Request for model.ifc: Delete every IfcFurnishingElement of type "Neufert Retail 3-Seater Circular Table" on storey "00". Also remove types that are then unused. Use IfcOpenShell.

First a look at what the model holds.

```python
import ifcopenshell
import ifcopenshell.util.element

model = ifcopenshell.open("model.ifc")
print(model.schema)
storey = next(s for s in model.by_type("IfcBuildingStorey") if s.Name == "00")
furniture = [e for e in ifcopenshell.util.element.get_decomposition(storey) if e.is_a("IfcFurnishingElement")]
seen = {}
for e in furniture:
    element_type = ifcopenshell.util.element.get_type(e)
    name = element_type.Name if element_type not in (None, e) else None
    seen[name] = seen.get(name, 0) + 1
for name, count in sorted(seen.items(), key=str):
    print(count, "x", name)
```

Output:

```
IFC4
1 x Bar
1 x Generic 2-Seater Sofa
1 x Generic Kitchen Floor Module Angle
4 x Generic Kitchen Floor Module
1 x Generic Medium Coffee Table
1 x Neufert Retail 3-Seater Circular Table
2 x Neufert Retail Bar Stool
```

```python
import ifcopenshell
import ifcopenshell.api.root
import ifcopenshell.util.element

model = ifcopenshell.open("model.ifc")

storey = next(s for s in model.by_type("IfcBuildingStorey") if s.Name == "00")
furniture = [e for e in ifcopenshell.util.element.get_decomposition(storey) if e.is_a("IfcFurnishingElement")]
targets = [e for e in furniture if (t := ifcopenshell.util.element.get_type(e)) not in (None, e) and t.Name == "Neufert Retail 3-Seater Circular Table"]
types = {ifcopenshell.util.element.get_type(e) for e in targets} - {None, *targets}

for e in targets:
    ifcopenshell.api.root.remove_product(model, product=e)
print(len(targets), "removed")

unused = [t for t in types if not ifcopenshell.util.element.get_types(t)]
for t in unused:
    ifcopenshell.api.root.remove_product(model, product=t)
print(len(unused), "unused types removed")

model.write("model_updated.ifc")
```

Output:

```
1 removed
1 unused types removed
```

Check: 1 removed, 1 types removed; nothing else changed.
